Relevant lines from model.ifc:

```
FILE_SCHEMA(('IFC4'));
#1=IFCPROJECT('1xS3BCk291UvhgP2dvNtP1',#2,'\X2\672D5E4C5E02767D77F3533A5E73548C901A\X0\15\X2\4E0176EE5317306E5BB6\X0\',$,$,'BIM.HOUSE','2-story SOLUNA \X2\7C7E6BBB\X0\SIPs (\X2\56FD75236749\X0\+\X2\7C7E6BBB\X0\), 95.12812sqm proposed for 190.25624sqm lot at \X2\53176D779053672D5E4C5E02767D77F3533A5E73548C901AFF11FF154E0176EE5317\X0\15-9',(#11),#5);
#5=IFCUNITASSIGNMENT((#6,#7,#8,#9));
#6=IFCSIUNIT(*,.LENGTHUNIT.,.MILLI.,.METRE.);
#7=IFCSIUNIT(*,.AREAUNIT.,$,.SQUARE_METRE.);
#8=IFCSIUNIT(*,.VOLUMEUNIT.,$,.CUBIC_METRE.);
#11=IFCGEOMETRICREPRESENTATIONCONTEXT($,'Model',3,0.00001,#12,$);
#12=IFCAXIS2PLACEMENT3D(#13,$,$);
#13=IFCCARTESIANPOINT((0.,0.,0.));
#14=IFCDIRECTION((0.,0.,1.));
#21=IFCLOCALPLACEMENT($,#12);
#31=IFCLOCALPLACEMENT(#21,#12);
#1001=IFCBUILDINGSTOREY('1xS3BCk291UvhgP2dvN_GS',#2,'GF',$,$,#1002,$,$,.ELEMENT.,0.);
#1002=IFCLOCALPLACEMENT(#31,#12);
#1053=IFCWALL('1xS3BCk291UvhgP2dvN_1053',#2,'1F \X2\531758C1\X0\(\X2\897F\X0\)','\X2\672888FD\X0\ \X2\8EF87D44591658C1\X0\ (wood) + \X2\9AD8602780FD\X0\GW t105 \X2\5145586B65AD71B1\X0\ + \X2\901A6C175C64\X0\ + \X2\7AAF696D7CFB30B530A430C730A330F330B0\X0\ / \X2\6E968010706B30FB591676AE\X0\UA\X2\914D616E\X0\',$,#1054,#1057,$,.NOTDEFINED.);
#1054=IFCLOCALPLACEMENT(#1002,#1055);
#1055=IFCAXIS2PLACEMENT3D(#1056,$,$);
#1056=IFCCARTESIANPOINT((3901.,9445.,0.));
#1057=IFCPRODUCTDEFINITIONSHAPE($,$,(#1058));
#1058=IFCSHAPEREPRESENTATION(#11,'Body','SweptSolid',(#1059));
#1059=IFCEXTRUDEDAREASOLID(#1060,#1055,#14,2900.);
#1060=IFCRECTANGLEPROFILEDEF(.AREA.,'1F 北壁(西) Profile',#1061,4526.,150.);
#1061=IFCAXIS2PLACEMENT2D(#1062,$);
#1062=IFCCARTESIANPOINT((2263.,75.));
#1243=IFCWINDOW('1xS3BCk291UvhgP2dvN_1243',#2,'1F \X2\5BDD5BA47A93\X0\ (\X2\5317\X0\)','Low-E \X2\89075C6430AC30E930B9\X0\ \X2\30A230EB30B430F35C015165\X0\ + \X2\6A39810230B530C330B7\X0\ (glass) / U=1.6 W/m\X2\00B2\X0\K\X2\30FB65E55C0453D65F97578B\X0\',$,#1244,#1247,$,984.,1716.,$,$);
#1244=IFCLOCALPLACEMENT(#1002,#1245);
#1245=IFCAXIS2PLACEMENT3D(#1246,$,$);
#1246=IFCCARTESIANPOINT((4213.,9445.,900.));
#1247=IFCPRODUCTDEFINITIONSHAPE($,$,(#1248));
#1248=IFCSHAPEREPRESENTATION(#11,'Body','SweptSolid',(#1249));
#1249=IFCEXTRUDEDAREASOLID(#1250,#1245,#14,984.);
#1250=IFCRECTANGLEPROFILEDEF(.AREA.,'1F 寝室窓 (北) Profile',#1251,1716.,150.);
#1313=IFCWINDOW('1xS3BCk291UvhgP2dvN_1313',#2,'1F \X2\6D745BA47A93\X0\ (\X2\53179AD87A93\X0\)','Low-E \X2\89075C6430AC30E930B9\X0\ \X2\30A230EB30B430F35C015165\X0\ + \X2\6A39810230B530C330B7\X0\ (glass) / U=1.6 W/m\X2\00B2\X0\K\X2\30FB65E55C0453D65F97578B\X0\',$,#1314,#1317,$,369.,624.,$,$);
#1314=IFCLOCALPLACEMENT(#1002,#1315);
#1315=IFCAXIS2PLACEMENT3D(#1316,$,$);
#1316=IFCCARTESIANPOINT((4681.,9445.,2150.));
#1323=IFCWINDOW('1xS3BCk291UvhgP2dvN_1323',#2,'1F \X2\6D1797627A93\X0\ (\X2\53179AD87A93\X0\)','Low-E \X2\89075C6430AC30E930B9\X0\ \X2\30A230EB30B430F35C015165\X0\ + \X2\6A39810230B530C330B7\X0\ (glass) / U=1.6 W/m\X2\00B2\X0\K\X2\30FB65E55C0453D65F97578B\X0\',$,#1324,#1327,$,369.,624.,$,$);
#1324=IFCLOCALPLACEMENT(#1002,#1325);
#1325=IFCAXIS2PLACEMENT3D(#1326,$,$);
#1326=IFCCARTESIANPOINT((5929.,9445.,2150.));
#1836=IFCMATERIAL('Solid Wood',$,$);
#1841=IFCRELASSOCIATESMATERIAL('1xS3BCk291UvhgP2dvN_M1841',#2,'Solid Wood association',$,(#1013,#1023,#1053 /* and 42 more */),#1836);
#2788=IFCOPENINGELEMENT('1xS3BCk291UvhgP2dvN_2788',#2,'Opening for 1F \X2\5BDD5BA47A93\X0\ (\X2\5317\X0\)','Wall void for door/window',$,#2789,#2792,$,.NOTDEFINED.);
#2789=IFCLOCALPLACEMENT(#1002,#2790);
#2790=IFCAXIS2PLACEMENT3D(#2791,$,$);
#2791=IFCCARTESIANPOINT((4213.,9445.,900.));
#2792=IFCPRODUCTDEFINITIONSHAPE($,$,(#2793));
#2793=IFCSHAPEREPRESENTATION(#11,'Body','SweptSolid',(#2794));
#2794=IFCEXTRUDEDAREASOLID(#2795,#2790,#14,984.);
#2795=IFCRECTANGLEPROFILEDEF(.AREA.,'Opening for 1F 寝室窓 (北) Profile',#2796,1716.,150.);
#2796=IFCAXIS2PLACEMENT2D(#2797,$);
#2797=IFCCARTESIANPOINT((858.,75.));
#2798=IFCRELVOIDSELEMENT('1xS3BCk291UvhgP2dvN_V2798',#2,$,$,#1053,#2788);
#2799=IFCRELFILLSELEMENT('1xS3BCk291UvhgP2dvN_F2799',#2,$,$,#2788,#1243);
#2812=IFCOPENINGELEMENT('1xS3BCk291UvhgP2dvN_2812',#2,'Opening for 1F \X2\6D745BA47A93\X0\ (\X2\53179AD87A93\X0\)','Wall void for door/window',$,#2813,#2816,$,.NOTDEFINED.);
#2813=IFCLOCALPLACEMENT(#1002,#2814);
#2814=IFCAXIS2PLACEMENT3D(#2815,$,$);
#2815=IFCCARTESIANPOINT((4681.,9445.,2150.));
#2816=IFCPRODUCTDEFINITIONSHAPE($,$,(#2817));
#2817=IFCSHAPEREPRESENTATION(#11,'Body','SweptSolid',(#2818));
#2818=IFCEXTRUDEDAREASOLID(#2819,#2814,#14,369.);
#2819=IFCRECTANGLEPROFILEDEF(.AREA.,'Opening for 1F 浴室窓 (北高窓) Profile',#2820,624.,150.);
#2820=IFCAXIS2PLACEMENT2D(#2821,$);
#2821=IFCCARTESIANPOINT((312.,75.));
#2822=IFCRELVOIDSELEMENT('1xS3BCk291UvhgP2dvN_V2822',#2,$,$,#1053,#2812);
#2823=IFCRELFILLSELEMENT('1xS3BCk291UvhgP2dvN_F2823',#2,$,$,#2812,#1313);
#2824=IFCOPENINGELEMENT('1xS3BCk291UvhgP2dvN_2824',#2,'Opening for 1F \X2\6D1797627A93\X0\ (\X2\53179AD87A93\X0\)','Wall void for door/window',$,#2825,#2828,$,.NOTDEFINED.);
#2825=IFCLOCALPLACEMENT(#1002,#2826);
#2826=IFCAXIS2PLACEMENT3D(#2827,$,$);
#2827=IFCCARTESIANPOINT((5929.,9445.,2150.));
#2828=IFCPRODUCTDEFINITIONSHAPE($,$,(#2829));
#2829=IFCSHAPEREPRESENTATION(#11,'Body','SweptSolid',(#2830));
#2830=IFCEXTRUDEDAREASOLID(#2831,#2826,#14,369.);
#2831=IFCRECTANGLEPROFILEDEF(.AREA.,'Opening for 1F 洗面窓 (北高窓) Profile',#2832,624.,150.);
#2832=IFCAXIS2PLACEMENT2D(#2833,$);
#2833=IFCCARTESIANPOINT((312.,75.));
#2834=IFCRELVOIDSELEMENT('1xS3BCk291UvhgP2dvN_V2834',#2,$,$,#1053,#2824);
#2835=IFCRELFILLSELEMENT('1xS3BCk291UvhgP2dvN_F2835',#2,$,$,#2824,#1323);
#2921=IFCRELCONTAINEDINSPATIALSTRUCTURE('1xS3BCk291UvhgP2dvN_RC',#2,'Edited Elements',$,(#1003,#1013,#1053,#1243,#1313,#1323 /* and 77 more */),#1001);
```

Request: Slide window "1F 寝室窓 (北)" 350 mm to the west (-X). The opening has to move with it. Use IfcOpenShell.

```python
import ifcopenshell
import ifcopenshell.api.geometry
import ifcopenshell.util.placement
import ifcopenshell.util.unit

model = ifcopenshell.open("model.ifc")
unit_scale = ifcopenshell.util.unit.calculate_unit_scale(model)

window = model.by_guid("1xS3BCk291UvhgP2dvN_1243")
opening = window.FillsVoids[0].RelatingOpeningElement
wall = opening.VoidsElements[0].RelatingBuildingElement

wall_matrix = ifcopenshell.util.placement.get_local_placement(wall.ObjectPlacement)
shift = wall_matrix[:3, 0] * -0.35 / unit_scale
before = ifcopenshell.util.placement.get_local_placement(window.ObjectPlacement)[:3, 3].copy()

# The window is not placed relative to its opening, so move both.
for product in (opening, window):
    matrix = ifcopenshell.util.placement.get_local_placement(product.ObjectPlacement)
    matrix[:3, 3] += shift
    ifcopenshell.api.geometry.edit_object_placement(model, product=product, matrix=matrix, is_si=False)

after = ifcopenshell.util.placement.get_local_placement(window.ObjectPlacement)[:3, 3]
print("window moved by", (after - before).round(3) + 0.0)

model.write("model-out.ifc")
```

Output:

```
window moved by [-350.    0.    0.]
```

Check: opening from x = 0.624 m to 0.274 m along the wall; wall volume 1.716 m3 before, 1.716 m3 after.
